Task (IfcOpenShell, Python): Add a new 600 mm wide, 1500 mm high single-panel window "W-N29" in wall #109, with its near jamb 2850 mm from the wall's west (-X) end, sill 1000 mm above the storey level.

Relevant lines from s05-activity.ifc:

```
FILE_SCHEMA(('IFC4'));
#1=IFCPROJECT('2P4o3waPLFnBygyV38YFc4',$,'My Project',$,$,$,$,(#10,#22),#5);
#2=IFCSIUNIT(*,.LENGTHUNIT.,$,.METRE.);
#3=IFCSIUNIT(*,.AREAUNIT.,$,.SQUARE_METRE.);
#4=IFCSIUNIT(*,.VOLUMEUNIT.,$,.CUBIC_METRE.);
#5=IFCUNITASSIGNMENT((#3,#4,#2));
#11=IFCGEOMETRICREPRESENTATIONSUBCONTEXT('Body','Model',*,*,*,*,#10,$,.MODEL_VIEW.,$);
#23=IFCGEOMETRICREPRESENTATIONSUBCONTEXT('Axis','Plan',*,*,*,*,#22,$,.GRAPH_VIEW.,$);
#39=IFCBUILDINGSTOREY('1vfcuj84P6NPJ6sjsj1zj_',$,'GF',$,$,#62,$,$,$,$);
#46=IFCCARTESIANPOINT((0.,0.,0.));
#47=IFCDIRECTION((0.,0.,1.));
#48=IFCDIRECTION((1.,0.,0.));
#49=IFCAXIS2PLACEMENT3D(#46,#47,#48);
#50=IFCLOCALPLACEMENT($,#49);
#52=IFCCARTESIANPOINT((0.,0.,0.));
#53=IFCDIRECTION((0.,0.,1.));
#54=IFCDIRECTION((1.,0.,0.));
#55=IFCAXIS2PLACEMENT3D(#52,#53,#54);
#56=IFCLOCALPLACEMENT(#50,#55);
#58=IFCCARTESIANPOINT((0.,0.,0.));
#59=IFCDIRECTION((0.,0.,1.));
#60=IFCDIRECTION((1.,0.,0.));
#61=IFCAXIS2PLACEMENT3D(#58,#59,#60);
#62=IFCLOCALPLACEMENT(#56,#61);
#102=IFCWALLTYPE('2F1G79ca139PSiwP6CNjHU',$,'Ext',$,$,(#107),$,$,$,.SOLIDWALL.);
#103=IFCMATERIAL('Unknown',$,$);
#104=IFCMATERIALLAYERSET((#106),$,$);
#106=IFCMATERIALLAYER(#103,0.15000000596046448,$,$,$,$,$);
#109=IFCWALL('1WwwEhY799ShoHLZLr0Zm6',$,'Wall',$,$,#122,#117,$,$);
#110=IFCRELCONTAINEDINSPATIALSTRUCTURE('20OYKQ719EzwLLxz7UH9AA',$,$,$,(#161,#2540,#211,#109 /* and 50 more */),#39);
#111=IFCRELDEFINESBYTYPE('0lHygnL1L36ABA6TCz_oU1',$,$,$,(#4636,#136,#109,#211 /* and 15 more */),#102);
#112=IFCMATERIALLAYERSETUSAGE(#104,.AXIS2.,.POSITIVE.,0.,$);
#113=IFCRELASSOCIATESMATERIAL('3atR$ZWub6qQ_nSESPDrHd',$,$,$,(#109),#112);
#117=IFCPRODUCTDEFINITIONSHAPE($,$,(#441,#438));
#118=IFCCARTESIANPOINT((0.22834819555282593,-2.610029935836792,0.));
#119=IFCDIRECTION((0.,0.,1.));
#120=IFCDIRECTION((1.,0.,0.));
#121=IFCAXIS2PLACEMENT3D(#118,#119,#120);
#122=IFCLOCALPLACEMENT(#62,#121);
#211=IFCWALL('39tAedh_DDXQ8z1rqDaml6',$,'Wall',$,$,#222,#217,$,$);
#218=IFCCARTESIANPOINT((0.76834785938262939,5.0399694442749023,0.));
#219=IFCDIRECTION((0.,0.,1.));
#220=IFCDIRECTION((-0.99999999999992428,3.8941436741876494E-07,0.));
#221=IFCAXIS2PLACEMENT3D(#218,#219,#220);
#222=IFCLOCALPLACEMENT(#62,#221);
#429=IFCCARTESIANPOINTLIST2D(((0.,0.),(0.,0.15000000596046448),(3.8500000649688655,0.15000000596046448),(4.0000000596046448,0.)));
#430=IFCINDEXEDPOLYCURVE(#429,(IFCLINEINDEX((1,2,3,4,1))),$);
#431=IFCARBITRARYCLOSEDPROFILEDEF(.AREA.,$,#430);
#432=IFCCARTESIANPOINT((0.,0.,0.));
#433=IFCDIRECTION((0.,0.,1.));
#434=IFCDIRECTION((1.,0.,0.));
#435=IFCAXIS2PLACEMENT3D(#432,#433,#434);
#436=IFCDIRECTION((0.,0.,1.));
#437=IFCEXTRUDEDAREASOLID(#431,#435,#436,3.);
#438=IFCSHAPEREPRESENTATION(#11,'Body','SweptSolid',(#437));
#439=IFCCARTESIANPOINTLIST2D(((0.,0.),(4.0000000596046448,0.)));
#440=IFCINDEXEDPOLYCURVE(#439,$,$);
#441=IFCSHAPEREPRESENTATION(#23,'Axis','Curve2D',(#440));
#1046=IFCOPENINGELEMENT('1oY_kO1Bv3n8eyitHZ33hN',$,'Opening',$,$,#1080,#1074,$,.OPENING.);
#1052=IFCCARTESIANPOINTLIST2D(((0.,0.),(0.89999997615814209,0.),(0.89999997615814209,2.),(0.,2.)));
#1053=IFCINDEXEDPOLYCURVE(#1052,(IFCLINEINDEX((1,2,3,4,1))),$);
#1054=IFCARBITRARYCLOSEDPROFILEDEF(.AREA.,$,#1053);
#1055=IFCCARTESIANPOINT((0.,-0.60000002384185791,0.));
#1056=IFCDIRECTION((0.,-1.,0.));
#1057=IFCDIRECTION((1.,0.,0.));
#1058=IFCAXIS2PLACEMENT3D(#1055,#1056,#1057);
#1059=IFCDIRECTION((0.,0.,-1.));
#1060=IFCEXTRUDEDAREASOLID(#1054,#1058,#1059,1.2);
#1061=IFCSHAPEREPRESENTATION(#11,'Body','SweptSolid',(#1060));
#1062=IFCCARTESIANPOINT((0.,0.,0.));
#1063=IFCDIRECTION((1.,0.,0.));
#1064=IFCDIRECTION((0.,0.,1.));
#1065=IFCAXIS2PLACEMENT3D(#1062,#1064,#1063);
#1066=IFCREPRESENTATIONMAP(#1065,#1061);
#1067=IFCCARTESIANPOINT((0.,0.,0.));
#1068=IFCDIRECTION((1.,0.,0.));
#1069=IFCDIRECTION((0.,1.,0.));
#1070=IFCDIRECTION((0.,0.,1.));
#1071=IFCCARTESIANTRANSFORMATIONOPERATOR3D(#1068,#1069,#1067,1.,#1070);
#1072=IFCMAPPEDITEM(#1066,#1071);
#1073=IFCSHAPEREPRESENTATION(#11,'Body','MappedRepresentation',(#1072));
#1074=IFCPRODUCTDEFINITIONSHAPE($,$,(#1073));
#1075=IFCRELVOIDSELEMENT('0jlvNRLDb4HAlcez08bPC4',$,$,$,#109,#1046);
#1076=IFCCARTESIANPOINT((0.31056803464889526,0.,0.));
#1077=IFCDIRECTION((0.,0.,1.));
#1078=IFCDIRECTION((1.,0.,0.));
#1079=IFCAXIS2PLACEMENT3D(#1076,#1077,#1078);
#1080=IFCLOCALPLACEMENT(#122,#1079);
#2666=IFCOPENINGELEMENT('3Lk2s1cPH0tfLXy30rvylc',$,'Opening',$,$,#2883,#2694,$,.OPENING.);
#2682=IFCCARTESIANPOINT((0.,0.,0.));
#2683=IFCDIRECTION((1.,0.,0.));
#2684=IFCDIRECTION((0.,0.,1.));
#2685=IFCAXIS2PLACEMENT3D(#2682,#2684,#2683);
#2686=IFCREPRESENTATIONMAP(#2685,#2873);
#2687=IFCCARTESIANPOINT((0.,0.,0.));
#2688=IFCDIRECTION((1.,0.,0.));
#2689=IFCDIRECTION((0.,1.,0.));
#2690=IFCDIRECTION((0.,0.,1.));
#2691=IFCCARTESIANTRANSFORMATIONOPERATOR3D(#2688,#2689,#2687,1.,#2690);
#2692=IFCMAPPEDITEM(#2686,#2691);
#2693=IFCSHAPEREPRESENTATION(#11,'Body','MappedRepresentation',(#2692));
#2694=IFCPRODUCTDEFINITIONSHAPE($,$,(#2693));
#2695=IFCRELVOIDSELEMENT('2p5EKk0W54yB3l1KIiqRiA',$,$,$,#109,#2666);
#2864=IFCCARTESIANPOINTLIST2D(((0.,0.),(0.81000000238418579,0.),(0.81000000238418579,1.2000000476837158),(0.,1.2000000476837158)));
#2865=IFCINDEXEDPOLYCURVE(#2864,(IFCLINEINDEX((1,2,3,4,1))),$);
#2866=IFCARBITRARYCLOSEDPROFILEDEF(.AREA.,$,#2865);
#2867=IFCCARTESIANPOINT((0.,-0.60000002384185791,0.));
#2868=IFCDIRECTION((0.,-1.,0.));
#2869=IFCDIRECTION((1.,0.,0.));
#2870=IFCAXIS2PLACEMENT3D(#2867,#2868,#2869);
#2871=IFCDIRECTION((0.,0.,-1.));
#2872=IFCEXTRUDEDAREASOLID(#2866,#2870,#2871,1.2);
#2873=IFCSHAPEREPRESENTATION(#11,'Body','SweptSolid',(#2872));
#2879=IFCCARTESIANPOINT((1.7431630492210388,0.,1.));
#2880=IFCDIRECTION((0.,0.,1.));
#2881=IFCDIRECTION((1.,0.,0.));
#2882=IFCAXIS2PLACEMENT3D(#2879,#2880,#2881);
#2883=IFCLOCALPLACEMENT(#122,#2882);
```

```python
import numpy as np
import ifcopenshell
import ifcopenshell.api.feature
import ifcopenshell.api.geometry
import ifcopenshell.api.root
import ifcopenshell.api.spatial
import ifcopenshell.geom
import ifcopenshell.util.element
import ifcopenshell.util.placement
import ifcopenshell.util.representation
import ifcopenshell.util.shape
import ifcopenshell.util.unit

model = ifcopenshell.open("s05-activity.ifc")
unit_scale = ifcopenshell.util.unit.calculate_unit_scale(model)
settings = ifcopenshell.geom.settings()


def volume(element):
    """Net volume in cubic metres, openings subtracted."""
    shape = ifcopenshell.geom.create_shape(settings, element)
    return ifcopenshell.util.shape.get_volume(shape.geometry)


wall = model.by_id(109)
storey = ifcopenshell.util.element.get_container(wall, ifc_class="IfcBuildingStorey")
context = ifcopenshell.util.representation.get_context(model, "Model", "Body", "MODEL_VIEW")
before = volume(wall)

width, height, from_end, sill = 0.6, 1.5, 2.85, 1  # metres

# The wall runs along its own X axis, and the end named is its -X end.
wall_shape = ifcopenshell.geom.create_shape(settings, wall)
x, y, z = ifcopenshell.util.shape.get_vertices(wall_shape.geometry).T
start = x.min() + from_end
face, thickness = float(y.min()), float(y.max() - y.min())
wall_matrix = ifcopenshell.util.placement.get_local_placement(wall.ObjectPlacement)
level = ifcopenshell.util.placement.get_local_placement(storey.ObjectPlacement)[2, 3]


def in_wall(x, y):
    """Placement at x, y metres in the wall's axes, at sill height."""
    matrix = wall_matrix.copy()
    matrix[:, 3] = wall_matrix @ np.array([x / unit_scale, y / unit_scale, 0.0, 1.0])
    matrix[2, 3] = level + sill / unit_scale
    return matrix


# Opening: a box that overshoots both wall faces by 50 mm.
opening = ifcopenshell.api.root.create_entity(model, ifc_class="IfcOpeningElement", predefined_type="OPENING")
box = ifcopenshell.api.geometry.add_wall_representation(
    model, context=context, length=width, height=height, thickness=thickness + 0.1
)
ifcopenshell.api.geometry.assign_representation(model, product=opening, representation=box)
ifcopenshell.api.geometry.edit_object_placement(model, product=opening, matrix=in_wall(start, face - 0.05), is_si=False)
ifcopenshell.api.feature.add_feature(model, feature=opening, element=wall)

window = ifcopenshell.api.root.create_entity(model, ifc_class="IfcWindow", name="W-N29", predefined_type="WINDOW")
window.OverallWidth, window.OverallHeight = width / unit_scale, height / unit_scale
window.PartitioningType = "SINGLE_PANEL"
body = ifcopenshell.api.geometry.add_window_representation(
    model,
    context=context,
    overall_width=window.OverallWidth,
    overall_height=window.OverallHeight,
    partition_type="SINGLE_PANEL",
)
ifcopenshell.api.geometry.assign_representation(model, product=window, representation=body)
ifcopenshell.api.spatial.assign_container(model, products=[window], relating_structure=storey)
ifcopenshell.api.feature.add_filling(model, opening=opening, element=window)

# Centre the window in the wall's thickness.
ifcopenshell.api.geometry.edit_object_placement(model, product=window, matrix=in_wall(start, face), is_si=False)
window_shape = ifcopenshell.geom.create_shape(settings, window)
depth = ifcopenshell.util.shape.get_vertices(window_shape.geometry)[:, 1]
offset = face + thickness / 2 - (depth.min() + depth.max()) / 2
ifcopenshell.api.geometry.edit_object_placement(model, product=window, matrix=in_wall(start, offset), is_si=False)

after = volume(wall)

print(f"wall volume {before:.3f} -> {after:.3f} m3")

model.write("s05-activity-out.ifc")
```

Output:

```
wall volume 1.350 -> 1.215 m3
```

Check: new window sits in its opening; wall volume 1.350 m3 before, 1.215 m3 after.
